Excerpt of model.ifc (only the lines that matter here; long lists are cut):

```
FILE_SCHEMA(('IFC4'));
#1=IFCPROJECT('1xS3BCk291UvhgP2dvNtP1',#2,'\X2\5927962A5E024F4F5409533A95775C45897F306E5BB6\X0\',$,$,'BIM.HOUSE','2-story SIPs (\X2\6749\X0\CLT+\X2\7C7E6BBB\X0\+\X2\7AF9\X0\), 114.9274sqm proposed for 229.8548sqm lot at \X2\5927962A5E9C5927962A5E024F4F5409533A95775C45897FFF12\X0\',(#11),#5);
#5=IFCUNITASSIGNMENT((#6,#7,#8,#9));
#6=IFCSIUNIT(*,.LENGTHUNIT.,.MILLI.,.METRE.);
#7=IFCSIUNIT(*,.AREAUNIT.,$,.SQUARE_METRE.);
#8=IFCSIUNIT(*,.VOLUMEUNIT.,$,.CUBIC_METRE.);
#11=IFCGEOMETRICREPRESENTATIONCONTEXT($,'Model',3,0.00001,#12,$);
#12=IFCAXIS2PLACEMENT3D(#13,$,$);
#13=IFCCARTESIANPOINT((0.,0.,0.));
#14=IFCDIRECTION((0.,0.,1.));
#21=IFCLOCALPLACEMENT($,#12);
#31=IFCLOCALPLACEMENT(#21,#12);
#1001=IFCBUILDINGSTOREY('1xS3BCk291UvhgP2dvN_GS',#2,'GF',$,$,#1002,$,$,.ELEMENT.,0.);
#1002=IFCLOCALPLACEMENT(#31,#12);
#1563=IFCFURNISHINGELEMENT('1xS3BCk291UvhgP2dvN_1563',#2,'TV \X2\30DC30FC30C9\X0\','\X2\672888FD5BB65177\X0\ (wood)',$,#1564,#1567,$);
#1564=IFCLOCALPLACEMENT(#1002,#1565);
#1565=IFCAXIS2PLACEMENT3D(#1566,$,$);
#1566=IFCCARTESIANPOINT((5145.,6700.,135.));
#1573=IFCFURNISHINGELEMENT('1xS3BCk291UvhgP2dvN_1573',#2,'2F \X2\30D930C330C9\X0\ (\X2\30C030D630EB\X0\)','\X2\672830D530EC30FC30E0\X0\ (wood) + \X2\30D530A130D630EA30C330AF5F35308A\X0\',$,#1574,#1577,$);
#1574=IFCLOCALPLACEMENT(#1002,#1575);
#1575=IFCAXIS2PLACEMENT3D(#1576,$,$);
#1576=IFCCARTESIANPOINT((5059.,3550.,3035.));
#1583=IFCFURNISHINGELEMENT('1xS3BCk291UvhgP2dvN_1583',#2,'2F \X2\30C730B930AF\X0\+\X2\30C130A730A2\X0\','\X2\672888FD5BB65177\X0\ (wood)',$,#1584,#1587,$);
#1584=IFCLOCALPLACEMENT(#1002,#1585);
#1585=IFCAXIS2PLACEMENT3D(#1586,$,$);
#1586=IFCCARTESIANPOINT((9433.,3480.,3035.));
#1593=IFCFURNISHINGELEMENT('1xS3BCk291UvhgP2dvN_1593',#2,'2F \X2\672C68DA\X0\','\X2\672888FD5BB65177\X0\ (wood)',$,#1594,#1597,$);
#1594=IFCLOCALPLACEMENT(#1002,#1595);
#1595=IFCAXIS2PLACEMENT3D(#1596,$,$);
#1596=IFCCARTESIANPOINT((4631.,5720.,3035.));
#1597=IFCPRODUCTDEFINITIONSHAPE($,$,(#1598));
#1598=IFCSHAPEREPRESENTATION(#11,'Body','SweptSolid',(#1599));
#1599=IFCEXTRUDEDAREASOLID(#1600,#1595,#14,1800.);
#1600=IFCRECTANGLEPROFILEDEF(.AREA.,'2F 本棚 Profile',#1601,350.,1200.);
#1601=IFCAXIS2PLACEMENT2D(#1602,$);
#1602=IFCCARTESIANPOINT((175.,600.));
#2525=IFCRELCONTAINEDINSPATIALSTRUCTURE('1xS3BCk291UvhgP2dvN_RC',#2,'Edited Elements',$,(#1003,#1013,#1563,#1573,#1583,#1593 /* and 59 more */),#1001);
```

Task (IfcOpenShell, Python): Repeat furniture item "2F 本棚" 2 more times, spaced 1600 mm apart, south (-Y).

```python
import numpy as np
import ifcopenshell
import ifcopenshell.api.geometry
import ifcopenshell.api.root
import ifcopenshell.util.element
import ifcopenshell.util.placement
import ifcopenshell.util.unit

model = ifcopenshell.open("model.ifc")
unit_scale = ifcopenshell.util.unit.calculate_unit_scale(model)


def reuse_history(source, copy):
    """copy_class also copies each property set's owner history, people and application; keep the originals."""
    for rel in copy.IsDefinedBy:
        if rel.is_a("IfcRelDefinesByProperties") and (history := rel.RelatingPropertyDefinition.OwnerHistory):
            rel.RelatingPropertyDefinition.OwnerHistory = source.OwnerHistory
            ifcopenshell.util.element.remove_deep2(model, history)


source = model.by_guid("1xS3BCk291UvhgP2dvN_1593")
base = ifcopenshell.util.placement.get_local_placement(source.ObjectPlacement)
step = np.array([0.0, -1.0, 0.0]) * 1.6 / unit_scale

for i in range(1, 3):
    copy = ifcopenshell.api.root.copy_class(model, product=source)
    copy.Representation = ifcopenshell.util.element.copy_deep(
        model, source.Representation, exclude=["IfcGeometricRepresentationContext", "IfcRepresentationMap"]
    )
    reuse_history(source, copy)
    matrix = base.copy()
    matrix[:3, 3] += i * step
    print("added at", matrix[:3, 3].round(3) + 0.0)
    ifcopenshell.api.geometry.edit_object_placement(model, product=copy, matrix=matrix, is_si=False)

model.write("model_edited.ifc")
```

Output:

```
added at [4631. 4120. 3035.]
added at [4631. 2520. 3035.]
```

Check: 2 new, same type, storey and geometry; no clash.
